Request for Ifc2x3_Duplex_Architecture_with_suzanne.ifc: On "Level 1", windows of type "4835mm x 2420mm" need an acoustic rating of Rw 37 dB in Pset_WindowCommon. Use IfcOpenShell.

First a look at what the model holds.

```python
import ifcopenshell
import ifcopenshell.util.element

model = ifcopenshell.open("Ifc2x3_Duplex_Architecture_with_suzanne.ifc")
print(model.schema)
storey = next(s for s in model.by_type("IfcBuildingStorey") if s.Name == "Level 1")
windows = [e for e in ifcopenshell.util.element.get_decomposition(storey) if e.is_a("IfcWindow")]
seen = {}
for e in windows:
    element_type = ifcopenshell.util.element.get_type(e)
    key = (element_type.Name if element_type != e and element_type else None, ifcopenshell.util.element.get_pset(e, "Pset_WindowCommon", "AcousticRating"))
    seen[key] = seen.get(key, 0) + 1
for (name, value), count in sorted(seen.items(), key=str):
    print(count, "x", name, "|", value)
```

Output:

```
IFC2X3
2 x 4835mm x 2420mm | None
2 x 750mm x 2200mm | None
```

```python
import ifcopenshell
import ifcopenshell.api.pset
import ifcopenshell.util.element

model = ifcopenshell.open("Ifc2x3_Duplex_Architecture_with_suzanne.ifc")

storey = next(s for s in model.by_type("IfcBuildingStorey") if s.Name == "Level 1")
windows = [e for e in ifcopenshell.util.element.get_decomposition(storey) if e.is_a("IfcWindow")]

count = 0
for e in windows:
    element_type = ifcopenshell.util.element.get_type(e)
    if element_type in (None, e) or element_type.Name != "4835mm x 2420mm":
        continue
    # add_pset returns the element's existing set when there is one.
    pset = ifcopenshell.api.pset.add_pset(model, product=e, name="Pset_WindowCommon")
    ifcopenshell.api.pset.edit_pset(model, pset=pset, properties={"AcousticRating": "Rw 37 dB"})
    count += 1

print(count, "windows updated")

model.write("Ifc2x3_Duplex_Architecture_with_suzanne_v2.ifc")
```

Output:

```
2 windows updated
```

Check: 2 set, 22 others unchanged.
